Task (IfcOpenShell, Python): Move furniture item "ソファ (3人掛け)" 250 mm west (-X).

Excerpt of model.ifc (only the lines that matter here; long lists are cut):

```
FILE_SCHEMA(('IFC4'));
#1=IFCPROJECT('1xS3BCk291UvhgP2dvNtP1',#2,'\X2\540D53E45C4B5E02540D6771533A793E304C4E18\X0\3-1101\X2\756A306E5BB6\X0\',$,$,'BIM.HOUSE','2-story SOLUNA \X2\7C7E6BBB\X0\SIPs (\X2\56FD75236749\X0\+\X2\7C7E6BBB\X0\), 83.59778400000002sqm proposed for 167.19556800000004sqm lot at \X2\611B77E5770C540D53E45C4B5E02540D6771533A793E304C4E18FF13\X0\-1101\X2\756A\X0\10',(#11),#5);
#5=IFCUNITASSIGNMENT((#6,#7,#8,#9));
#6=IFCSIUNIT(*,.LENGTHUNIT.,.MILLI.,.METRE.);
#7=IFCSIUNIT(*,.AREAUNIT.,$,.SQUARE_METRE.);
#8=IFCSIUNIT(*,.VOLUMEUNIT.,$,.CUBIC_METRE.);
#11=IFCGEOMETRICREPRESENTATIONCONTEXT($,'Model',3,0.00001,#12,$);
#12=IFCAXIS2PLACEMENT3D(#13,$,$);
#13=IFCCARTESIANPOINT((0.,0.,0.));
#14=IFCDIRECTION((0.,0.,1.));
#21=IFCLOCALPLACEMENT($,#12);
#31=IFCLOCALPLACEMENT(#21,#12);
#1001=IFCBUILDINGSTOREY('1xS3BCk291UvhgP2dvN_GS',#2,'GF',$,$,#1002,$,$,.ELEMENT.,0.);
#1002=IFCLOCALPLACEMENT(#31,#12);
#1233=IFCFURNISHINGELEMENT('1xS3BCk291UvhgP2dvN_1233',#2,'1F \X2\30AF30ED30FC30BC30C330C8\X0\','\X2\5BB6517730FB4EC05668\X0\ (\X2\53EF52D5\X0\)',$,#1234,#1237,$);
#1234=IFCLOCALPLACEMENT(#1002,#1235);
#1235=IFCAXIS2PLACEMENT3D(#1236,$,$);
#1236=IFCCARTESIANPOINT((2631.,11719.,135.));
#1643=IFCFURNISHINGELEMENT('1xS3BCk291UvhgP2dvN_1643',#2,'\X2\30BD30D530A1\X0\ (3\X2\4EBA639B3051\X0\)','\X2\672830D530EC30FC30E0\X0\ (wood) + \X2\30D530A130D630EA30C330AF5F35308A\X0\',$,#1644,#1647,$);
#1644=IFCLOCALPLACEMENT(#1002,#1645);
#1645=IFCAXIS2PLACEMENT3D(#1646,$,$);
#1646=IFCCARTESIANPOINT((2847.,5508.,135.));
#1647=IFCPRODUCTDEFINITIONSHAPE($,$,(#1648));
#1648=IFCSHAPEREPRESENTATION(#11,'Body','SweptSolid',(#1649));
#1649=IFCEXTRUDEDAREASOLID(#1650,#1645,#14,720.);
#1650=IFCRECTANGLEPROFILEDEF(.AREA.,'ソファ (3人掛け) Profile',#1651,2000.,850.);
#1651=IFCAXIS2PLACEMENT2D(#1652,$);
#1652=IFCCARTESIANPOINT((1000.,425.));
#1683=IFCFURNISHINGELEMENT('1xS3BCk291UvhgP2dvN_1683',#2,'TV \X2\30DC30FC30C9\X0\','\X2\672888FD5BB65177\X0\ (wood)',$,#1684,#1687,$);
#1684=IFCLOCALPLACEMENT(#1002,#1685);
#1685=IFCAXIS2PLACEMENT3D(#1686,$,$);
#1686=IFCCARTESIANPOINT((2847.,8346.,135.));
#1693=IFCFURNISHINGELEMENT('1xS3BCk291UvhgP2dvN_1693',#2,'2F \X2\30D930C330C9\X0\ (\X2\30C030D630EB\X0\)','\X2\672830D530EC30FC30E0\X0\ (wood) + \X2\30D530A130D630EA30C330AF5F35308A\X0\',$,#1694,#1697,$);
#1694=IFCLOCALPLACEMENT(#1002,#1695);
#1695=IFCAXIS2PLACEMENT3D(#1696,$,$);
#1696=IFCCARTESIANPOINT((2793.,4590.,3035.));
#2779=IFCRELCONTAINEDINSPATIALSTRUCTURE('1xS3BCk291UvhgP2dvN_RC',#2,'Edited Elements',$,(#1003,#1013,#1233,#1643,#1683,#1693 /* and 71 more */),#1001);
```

```python
import ifcopenshell
import ifcopenshell.api.geometry
import ifcopenshell.util.placement

model = ifcopenshell.open("model.ifc")

item = model.by_guid("1xS3BCk291UvhgP2dvN_1643")
matrix = ifcopenshell.util.placement.get_local_placement(item.ObjectPlacement)
matrix[0, 3] -= 250.0
ifcopenshell.api.geometry.edit_object_placement(model, product=item, matrix=matrix, is_si=False)

print(ifcopenshell.util.placement.get_local_placement(item.ObjectPlacement).round(3) + 0.0)

model.write("model_updated.ifc")
```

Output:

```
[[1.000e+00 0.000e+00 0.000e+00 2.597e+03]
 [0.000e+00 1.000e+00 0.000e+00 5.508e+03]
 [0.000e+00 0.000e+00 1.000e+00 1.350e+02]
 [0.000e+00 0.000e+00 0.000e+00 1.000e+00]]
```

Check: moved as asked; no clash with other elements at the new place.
